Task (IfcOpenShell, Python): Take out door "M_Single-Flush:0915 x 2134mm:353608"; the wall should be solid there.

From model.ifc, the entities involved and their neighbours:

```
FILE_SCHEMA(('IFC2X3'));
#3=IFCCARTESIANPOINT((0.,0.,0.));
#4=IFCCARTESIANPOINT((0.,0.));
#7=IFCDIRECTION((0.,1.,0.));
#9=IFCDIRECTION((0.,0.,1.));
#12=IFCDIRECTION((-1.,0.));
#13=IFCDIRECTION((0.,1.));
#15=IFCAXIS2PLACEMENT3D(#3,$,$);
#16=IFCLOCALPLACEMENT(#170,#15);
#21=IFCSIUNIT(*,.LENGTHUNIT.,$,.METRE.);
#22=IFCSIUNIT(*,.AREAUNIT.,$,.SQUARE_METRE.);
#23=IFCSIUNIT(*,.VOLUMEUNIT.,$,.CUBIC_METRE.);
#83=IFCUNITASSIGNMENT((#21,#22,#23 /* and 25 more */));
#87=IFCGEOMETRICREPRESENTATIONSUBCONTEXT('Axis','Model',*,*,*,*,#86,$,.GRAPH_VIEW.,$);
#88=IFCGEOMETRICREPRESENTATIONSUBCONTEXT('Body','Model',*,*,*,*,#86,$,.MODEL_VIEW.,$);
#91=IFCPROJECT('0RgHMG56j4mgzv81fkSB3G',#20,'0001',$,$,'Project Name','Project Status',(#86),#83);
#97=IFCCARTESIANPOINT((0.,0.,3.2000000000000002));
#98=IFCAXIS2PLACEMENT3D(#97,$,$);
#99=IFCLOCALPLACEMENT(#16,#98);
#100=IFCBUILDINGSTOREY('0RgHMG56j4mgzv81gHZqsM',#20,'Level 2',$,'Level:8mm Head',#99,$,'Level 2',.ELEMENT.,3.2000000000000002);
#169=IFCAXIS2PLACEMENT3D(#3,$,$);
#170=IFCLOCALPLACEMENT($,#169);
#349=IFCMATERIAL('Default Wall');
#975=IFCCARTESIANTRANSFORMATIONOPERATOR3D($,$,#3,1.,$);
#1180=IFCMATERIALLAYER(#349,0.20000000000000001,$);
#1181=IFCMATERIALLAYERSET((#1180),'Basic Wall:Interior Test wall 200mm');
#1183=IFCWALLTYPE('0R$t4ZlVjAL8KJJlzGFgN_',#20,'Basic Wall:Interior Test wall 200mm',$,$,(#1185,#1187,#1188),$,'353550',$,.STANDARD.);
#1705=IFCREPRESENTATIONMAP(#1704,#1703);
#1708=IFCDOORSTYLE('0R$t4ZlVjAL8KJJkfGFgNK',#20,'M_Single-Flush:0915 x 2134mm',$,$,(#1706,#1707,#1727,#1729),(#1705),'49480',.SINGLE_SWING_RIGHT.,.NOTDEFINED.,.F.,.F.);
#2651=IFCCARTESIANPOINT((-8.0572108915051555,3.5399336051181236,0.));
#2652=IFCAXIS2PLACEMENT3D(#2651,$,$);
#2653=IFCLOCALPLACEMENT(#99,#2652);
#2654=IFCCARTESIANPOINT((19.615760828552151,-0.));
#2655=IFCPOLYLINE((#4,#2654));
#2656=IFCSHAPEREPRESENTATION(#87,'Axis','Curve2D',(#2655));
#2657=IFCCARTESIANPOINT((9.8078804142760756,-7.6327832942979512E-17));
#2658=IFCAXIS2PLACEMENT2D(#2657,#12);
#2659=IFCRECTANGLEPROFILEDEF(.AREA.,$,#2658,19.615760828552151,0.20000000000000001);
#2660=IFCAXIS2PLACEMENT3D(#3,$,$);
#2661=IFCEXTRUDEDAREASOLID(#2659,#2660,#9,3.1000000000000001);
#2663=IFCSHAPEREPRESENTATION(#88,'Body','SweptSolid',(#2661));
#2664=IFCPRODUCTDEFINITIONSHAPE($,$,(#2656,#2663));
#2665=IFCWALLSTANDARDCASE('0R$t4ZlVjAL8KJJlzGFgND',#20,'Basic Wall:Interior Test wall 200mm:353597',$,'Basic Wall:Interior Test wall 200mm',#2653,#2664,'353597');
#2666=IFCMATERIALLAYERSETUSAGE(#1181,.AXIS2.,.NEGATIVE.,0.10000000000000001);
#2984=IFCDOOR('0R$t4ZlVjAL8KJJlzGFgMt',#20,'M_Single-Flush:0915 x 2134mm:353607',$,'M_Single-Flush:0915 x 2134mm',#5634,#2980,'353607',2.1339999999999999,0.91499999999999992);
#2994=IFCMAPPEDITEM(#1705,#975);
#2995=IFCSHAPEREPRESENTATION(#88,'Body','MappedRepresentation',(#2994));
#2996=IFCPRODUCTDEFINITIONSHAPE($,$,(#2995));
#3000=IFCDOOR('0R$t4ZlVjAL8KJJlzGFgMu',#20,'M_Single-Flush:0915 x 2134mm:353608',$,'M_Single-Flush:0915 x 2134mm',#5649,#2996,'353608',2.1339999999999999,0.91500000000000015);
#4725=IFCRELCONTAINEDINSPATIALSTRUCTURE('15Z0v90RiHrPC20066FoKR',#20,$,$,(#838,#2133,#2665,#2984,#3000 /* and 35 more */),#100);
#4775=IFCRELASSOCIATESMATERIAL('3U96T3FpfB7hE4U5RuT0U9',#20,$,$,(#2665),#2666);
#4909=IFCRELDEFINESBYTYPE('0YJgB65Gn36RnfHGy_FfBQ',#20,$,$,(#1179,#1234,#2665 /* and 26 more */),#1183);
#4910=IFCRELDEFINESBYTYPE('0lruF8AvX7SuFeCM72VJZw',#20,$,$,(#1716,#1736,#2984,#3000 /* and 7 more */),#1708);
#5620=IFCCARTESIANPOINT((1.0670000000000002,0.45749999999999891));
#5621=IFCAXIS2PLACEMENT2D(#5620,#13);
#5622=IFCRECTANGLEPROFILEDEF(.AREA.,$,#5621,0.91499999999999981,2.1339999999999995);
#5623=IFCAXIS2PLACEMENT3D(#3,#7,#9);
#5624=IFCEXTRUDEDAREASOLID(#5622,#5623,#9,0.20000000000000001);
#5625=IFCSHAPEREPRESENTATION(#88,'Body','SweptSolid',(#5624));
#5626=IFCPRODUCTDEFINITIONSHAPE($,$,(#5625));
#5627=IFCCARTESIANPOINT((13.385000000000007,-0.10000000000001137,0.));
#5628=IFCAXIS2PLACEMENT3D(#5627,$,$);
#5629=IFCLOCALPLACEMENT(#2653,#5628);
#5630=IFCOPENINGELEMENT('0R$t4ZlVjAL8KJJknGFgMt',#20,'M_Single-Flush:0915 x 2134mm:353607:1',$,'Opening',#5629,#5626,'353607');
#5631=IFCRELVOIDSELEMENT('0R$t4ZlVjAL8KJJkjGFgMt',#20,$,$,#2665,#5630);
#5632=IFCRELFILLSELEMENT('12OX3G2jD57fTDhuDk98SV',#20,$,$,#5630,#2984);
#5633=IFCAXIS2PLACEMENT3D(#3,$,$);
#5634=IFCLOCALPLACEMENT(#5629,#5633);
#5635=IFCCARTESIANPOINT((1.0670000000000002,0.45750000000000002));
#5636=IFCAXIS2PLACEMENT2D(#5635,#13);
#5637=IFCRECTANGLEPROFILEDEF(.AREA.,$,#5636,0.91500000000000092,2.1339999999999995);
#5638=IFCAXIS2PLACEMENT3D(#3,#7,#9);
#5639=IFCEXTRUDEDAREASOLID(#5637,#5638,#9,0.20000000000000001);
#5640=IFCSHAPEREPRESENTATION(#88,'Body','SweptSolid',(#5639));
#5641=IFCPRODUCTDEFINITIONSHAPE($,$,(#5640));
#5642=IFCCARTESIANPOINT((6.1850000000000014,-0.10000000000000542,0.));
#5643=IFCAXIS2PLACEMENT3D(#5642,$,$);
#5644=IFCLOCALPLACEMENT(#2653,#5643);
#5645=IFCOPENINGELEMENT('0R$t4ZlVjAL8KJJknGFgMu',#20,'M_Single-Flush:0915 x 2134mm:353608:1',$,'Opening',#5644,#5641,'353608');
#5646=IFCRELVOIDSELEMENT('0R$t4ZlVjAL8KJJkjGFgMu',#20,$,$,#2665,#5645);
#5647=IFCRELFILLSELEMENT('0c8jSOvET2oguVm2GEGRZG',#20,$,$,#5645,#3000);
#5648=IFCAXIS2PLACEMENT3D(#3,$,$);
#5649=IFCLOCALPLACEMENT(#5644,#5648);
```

```python
import ifcopenshell
import ifcopenshell.api.feature
import ifcopenshell.api.root
import ifcopenshell.geom
import ifcopenshell.util.shape

model = ifcopenshell.open("model.ifc")
settings = ifcopenshell.geom.settings()


def volume(element):
    """Net volume in cubic metres, openings subtracted."""
    shape = ifcopenshell.geom.create_shape(settings, element)
    return ifcopenshell.util.shape.get_volume(shape.geometry)


door = model.by_guid("0R$t4ZlVjAL8KJJlzGFgMu")
opening = door.FillsVoids[0].RelatingOpeningElement
wall = opening.VoidsElements[0].RelatingBuildingElement
before = volume(wall)

ifcopenshell.api.root.remove_product(model, product=door)
ifcopenshell.api.feature.remove_feature(model, feature=opening)

after = volume(wall)

print(f"wall volume {before:.3f} -> {after:.3f} m3")

model.write("model-out.ifc")
```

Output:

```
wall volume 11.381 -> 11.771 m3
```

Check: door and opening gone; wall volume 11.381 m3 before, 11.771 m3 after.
